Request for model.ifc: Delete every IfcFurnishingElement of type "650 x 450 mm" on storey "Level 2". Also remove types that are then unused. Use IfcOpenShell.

First a look at what the model holds.

```python
import ifcopenshell
import ifcopenshell.util.element

model = ifcopenshell.open("model.ifc")
print(model.schema)
storey = next(s for s in model.by_type("IfcBuildingStorey") if s.Name == "Level 2")
furniture = [e for e in ifcopenshell.util.element.get_decomposition(storey) if e.is_a("IfcFurnishingElement")]
seen = {}
for e in furniture:
    element_type = ifcopenshell.util.element.get_type(e)
    name = element_type.Name if element_type not in (None, e) else None
    seen[name] = seen.get(name, 0) + 1
for name, count in sorted(seen.items(), key=str):
    print(count, "x", name)
```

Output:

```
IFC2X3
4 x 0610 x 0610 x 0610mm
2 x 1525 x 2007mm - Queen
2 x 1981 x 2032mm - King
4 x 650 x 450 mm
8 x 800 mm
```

```python
import ifcopenshell
import ifcopenshell.api.root
import ifcopenshell.util.element

model = ifcopenshell.open("model.ifc")

storey = next(s for s in model.by_type("IfcBuildingStorey") if s.Name == "Level 2")
furniture = [e for e in ifcopenshell.util.element.get_decomposition(storey) if e.is_a("IfcFurnishingElement")]
targets = [e for e in furniture if (t := ifcopenshell.util.element.get_type(e)) not in (None, e) and t.Name == "650 x 450 mm"]
types = {ifcopenshell.util.element.get_type(e) for e in targets} - {None, *targets}

for e in targets:
    ifcopenshell.api.root.remove_product(model, product=e)
print(len(targets), "removed")

unused = [t for t in types if not ifcopenshell.util.element.get_types(t)]
for t in unused:
    ifcopenshell.api.root.remove_product(model, product=t)
print(len(unused), "unused types removed")

model.write("model-out.ifc")
```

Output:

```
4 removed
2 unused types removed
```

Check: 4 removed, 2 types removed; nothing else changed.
